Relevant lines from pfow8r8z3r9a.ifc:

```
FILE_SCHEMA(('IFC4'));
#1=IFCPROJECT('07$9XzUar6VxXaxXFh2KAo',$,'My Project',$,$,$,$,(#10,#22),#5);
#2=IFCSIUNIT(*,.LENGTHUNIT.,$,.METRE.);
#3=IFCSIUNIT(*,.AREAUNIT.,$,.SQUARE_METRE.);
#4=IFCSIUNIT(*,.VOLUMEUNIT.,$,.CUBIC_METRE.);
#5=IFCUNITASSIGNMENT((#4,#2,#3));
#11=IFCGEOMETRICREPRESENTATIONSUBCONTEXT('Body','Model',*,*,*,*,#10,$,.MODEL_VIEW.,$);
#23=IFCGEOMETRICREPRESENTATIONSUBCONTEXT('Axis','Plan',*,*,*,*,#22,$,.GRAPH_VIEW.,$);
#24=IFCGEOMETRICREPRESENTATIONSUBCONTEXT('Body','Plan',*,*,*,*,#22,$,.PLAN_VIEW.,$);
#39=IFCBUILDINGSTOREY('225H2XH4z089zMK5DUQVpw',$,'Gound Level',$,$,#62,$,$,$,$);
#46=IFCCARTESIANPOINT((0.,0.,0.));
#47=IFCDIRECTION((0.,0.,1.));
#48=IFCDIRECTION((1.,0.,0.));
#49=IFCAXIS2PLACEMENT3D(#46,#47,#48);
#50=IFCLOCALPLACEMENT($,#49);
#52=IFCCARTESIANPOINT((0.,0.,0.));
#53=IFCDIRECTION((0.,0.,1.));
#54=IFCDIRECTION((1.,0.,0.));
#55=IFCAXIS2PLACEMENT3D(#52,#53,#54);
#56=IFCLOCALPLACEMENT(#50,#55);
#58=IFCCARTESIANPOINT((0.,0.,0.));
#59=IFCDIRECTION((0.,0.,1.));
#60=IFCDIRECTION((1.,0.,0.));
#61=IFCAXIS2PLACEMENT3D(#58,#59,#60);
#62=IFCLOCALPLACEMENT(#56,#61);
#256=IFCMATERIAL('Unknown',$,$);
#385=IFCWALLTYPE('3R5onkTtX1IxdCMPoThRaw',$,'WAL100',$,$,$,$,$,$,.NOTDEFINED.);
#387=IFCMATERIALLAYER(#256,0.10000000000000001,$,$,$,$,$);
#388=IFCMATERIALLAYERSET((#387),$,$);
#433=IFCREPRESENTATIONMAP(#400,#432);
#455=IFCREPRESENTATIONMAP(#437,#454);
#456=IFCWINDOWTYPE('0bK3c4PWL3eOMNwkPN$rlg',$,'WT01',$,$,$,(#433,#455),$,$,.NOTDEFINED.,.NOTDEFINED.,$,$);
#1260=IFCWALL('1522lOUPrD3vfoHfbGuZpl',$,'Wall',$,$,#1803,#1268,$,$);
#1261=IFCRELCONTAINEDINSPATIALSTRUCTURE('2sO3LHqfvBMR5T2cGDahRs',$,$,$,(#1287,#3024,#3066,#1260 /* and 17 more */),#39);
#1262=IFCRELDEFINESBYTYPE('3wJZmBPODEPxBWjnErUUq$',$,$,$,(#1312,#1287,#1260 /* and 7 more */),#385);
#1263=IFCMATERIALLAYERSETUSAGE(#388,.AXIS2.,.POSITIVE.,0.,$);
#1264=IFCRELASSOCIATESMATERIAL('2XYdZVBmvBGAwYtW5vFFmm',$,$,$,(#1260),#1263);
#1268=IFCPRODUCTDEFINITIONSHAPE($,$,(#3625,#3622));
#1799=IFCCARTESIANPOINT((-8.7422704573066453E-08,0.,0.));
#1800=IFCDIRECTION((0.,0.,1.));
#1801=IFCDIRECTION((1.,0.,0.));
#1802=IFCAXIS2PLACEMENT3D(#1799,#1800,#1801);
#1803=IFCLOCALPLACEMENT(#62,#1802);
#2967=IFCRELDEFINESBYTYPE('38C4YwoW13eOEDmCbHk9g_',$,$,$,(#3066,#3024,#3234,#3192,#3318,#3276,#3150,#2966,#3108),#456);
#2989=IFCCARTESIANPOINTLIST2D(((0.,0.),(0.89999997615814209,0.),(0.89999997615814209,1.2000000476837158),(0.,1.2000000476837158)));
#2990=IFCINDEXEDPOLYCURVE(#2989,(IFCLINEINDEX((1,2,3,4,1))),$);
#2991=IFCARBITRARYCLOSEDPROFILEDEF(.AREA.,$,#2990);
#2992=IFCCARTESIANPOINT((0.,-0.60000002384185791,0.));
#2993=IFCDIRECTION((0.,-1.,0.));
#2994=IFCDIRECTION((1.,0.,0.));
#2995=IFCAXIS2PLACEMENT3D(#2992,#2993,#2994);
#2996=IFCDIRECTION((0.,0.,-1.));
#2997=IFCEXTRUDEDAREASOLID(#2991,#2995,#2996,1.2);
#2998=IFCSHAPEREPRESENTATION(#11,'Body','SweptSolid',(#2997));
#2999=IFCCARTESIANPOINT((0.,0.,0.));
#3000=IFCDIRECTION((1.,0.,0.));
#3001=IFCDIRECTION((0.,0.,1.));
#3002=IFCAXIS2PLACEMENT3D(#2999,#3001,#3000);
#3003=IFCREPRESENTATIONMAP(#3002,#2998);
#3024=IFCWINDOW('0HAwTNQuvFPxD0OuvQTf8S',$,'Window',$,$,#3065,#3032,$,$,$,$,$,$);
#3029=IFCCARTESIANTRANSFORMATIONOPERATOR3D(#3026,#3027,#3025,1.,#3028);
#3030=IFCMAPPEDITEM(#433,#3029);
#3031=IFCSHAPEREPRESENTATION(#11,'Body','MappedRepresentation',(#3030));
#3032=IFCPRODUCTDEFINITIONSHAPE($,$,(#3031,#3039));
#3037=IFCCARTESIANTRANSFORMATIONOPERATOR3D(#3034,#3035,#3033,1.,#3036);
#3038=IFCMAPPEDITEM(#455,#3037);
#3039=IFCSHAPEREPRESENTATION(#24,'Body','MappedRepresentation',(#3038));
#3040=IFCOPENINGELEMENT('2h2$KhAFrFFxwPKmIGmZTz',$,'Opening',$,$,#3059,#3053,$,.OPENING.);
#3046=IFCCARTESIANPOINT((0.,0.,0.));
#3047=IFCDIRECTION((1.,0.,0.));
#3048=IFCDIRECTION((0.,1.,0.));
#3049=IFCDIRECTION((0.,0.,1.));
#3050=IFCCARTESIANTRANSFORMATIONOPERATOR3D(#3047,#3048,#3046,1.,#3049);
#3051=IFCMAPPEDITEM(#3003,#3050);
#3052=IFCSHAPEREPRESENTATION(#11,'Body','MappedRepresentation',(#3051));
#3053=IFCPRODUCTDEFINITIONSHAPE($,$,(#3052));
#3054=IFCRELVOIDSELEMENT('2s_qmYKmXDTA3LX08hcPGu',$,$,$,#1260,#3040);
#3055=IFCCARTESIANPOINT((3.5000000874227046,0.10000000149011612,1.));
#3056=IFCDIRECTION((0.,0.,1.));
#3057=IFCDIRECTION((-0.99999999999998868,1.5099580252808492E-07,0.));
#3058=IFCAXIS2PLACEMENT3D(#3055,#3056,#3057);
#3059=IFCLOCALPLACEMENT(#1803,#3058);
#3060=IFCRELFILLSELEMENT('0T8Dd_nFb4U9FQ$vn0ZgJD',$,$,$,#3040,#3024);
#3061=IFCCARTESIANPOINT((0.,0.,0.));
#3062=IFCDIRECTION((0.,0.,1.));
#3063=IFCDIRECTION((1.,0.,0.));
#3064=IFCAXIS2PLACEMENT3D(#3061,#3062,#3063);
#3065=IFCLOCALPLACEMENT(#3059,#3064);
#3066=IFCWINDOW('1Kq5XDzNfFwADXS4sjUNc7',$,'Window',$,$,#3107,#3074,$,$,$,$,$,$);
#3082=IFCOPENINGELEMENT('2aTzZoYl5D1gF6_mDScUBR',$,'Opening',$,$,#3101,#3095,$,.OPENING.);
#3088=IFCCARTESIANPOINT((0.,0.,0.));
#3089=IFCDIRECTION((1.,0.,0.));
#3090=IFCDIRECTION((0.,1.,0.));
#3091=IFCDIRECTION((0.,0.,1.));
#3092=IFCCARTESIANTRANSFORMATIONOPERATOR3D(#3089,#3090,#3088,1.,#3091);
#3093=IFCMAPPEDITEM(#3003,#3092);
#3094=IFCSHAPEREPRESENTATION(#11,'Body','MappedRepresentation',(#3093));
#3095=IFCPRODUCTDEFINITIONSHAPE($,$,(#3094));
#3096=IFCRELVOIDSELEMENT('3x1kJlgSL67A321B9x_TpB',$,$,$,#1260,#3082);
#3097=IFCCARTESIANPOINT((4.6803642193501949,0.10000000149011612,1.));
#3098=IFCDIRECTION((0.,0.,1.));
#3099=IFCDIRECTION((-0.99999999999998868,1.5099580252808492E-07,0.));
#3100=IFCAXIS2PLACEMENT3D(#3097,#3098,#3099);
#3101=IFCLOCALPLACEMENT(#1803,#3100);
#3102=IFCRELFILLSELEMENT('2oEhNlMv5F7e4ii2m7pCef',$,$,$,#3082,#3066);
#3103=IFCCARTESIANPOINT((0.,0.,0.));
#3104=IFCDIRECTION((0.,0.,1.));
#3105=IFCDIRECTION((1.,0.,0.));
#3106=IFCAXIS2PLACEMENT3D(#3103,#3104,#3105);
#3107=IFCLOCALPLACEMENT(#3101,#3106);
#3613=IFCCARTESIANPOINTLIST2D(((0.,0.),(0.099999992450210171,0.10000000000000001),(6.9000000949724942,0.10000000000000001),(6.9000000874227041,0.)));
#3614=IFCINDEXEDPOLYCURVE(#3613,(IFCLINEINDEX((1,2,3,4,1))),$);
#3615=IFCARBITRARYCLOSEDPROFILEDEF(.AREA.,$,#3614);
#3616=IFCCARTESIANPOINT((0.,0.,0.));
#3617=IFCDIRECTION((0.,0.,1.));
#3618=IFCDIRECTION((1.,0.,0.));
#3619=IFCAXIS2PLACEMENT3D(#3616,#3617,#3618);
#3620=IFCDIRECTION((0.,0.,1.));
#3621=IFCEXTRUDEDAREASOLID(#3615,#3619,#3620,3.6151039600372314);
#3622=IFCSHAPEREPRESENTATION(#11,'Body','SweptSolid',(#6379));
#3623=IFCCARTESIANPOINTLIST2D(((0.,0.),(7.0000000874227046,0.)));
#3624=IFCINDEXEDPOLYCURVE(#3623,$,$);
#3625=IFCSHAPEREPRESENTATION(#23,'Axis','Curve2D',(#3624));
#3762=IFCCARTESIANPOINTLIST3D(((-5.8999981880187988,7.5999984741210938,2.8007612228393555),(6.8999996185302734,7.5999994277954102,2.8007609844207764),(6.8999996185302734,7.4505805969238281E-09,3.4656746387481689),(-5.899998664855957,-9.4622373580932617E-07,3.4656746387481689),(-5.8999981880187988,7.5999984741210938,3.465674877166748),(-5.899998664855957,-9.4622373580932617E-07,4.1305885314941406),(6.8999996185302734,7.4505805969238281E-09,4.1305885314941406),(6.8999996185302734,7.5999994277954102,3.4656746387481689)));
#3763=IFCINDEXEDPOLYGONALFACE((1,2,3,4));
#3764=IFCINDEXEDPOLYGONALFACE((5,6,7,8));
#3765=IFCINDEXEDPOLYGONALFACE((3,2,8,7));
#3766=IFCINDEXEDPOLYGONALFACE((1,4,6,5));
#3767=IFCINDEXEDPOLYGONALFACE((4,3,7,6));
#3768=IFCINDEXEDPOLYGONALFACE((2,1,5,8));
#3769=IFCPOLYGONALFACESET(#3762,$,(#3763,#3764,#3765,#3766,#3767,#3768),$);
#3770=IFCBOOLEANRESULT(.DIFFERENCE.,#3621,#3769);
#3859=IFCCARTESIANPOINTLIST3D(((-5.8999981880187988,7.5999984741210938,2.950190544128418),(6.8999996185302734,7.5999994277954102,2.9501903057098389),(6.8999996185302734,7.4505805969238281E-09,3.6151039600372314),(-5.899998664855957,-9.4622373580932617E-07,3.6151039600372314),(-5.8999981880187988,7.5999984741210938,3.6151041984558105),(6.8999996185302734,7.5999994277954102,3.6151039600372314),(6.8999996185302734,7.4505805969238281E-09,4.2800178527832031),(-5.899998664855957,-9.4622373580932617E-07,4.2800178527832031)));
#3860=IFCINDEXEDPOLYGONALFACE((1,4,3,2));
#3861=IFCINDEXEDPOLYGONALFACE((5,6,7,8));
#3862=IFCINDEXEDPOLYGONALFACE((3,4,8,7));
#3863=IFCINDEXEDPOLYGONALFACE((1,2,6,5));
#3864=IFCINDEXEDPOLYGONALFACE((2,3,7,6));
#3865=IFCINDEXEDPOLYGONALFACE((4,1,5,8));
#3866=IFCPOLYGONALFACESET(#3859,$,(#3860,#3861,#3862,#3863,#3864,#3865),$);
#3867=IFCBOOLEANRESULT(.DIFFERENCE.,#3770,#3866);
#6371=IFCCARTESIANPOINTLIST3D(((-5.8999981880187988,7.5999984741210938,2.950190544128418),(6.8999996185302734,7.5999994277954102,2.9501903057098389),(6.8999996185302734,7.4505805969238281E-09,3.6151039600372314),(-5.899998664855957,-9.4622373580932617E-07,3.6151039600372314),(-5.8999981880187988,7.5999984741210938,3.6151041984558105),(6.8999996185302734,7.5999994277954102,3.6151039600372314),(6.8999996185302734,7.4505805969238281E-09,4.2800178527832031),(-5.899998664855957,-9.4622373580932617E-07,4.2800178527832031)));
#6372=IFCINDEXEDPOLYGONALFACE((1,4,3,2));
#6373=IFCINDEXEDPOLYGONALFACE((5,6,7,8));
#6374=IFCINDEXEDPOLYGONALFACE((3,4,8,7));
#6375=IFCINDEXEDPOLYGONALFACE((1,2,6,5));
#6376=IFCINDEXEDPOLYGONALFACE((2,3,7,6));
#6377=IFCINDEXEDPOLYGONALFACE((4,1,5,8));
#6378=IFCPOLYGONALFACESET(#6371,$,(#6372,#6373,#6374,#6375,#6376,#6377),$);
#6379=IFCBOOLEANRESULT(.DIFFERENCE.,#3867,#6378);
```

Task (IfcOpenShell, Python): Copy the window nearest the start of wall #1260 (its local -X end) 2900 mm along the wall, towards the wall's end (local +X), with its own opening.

```python
import ifcopenshell
import ifcopenshell.api.feature
import ifcopenshell.api.geometry
import ifcopenshell.api.root
import ifcopenshell.geom
import ifcopenshell.util.element
import ifcopenshell.util.placement
import ifcopenshell.util.shape

model = ifcopenshell.open("pfow8r8z3r9a.ifc")
settings = ifcopenshell.geom.settings()


def volume(element):
    """Net volume in cubic metres, openings subtracted."""
    shape = ifcopenshell.geom.create_shape(settings, element)
    return ifcopenshell.util.shape.get_volume(shape.geometry)


window = model.by_guid("0HAwTNQuvFPxD0OuvQTf8S")
opening = window.FillsVoids[0].RelatingOpeningElement
wall = opening.VoidsElements[0].RelatingBuildingElement
before = volume(wall)
shift = ifcopenshell.util.placement.get_local_placement(wall.ObjectPlacement)[:3, 0] * 2.9

# copy_class copies the void relationship, type, container and properties, but no geometry.
new_opening = ifcopenshell.api.root.copy_class(model, product=opening)
new_opening.Representation = ifcopenshell.util.element.copy_deep(
    model, opening.Representation, exclude=["IfcGeometricRepresentationContext", "IfcRepresentationMap"]
)
new_window = ifcopenshell.api.root.copy_class(model, product=window)
new_window.Representation = ifcopenshell.util.element.copy_deep(
    model, window.Representation, exclude=["IfcGeometricRepresentationContext", "IfcRepresentationMap"]
)
ifcopenshell.api.feature.add_filling(model, opening=new_opening, element=new_window)

for old, new in ((opening, new_opening), (window, new_window)):
    matrix = ifcopenshell.util.placement.get_local_placement(old.ObjectPlacement)
    matrix[:3, 3] += shift
    ifcopenshell.api.geometry.edit_object_placement(model, product=new, matrix=matrix, is_si=False)

after = volume(wall)

print(f"wall volume {before:.3f} -> {after:.3f} m3")

model.write("pfow8r8z3r9a_v2.ifc")
```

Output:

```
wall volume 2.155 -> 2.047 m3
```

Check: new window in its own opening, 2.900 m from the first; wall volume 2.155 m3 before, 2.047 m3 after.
